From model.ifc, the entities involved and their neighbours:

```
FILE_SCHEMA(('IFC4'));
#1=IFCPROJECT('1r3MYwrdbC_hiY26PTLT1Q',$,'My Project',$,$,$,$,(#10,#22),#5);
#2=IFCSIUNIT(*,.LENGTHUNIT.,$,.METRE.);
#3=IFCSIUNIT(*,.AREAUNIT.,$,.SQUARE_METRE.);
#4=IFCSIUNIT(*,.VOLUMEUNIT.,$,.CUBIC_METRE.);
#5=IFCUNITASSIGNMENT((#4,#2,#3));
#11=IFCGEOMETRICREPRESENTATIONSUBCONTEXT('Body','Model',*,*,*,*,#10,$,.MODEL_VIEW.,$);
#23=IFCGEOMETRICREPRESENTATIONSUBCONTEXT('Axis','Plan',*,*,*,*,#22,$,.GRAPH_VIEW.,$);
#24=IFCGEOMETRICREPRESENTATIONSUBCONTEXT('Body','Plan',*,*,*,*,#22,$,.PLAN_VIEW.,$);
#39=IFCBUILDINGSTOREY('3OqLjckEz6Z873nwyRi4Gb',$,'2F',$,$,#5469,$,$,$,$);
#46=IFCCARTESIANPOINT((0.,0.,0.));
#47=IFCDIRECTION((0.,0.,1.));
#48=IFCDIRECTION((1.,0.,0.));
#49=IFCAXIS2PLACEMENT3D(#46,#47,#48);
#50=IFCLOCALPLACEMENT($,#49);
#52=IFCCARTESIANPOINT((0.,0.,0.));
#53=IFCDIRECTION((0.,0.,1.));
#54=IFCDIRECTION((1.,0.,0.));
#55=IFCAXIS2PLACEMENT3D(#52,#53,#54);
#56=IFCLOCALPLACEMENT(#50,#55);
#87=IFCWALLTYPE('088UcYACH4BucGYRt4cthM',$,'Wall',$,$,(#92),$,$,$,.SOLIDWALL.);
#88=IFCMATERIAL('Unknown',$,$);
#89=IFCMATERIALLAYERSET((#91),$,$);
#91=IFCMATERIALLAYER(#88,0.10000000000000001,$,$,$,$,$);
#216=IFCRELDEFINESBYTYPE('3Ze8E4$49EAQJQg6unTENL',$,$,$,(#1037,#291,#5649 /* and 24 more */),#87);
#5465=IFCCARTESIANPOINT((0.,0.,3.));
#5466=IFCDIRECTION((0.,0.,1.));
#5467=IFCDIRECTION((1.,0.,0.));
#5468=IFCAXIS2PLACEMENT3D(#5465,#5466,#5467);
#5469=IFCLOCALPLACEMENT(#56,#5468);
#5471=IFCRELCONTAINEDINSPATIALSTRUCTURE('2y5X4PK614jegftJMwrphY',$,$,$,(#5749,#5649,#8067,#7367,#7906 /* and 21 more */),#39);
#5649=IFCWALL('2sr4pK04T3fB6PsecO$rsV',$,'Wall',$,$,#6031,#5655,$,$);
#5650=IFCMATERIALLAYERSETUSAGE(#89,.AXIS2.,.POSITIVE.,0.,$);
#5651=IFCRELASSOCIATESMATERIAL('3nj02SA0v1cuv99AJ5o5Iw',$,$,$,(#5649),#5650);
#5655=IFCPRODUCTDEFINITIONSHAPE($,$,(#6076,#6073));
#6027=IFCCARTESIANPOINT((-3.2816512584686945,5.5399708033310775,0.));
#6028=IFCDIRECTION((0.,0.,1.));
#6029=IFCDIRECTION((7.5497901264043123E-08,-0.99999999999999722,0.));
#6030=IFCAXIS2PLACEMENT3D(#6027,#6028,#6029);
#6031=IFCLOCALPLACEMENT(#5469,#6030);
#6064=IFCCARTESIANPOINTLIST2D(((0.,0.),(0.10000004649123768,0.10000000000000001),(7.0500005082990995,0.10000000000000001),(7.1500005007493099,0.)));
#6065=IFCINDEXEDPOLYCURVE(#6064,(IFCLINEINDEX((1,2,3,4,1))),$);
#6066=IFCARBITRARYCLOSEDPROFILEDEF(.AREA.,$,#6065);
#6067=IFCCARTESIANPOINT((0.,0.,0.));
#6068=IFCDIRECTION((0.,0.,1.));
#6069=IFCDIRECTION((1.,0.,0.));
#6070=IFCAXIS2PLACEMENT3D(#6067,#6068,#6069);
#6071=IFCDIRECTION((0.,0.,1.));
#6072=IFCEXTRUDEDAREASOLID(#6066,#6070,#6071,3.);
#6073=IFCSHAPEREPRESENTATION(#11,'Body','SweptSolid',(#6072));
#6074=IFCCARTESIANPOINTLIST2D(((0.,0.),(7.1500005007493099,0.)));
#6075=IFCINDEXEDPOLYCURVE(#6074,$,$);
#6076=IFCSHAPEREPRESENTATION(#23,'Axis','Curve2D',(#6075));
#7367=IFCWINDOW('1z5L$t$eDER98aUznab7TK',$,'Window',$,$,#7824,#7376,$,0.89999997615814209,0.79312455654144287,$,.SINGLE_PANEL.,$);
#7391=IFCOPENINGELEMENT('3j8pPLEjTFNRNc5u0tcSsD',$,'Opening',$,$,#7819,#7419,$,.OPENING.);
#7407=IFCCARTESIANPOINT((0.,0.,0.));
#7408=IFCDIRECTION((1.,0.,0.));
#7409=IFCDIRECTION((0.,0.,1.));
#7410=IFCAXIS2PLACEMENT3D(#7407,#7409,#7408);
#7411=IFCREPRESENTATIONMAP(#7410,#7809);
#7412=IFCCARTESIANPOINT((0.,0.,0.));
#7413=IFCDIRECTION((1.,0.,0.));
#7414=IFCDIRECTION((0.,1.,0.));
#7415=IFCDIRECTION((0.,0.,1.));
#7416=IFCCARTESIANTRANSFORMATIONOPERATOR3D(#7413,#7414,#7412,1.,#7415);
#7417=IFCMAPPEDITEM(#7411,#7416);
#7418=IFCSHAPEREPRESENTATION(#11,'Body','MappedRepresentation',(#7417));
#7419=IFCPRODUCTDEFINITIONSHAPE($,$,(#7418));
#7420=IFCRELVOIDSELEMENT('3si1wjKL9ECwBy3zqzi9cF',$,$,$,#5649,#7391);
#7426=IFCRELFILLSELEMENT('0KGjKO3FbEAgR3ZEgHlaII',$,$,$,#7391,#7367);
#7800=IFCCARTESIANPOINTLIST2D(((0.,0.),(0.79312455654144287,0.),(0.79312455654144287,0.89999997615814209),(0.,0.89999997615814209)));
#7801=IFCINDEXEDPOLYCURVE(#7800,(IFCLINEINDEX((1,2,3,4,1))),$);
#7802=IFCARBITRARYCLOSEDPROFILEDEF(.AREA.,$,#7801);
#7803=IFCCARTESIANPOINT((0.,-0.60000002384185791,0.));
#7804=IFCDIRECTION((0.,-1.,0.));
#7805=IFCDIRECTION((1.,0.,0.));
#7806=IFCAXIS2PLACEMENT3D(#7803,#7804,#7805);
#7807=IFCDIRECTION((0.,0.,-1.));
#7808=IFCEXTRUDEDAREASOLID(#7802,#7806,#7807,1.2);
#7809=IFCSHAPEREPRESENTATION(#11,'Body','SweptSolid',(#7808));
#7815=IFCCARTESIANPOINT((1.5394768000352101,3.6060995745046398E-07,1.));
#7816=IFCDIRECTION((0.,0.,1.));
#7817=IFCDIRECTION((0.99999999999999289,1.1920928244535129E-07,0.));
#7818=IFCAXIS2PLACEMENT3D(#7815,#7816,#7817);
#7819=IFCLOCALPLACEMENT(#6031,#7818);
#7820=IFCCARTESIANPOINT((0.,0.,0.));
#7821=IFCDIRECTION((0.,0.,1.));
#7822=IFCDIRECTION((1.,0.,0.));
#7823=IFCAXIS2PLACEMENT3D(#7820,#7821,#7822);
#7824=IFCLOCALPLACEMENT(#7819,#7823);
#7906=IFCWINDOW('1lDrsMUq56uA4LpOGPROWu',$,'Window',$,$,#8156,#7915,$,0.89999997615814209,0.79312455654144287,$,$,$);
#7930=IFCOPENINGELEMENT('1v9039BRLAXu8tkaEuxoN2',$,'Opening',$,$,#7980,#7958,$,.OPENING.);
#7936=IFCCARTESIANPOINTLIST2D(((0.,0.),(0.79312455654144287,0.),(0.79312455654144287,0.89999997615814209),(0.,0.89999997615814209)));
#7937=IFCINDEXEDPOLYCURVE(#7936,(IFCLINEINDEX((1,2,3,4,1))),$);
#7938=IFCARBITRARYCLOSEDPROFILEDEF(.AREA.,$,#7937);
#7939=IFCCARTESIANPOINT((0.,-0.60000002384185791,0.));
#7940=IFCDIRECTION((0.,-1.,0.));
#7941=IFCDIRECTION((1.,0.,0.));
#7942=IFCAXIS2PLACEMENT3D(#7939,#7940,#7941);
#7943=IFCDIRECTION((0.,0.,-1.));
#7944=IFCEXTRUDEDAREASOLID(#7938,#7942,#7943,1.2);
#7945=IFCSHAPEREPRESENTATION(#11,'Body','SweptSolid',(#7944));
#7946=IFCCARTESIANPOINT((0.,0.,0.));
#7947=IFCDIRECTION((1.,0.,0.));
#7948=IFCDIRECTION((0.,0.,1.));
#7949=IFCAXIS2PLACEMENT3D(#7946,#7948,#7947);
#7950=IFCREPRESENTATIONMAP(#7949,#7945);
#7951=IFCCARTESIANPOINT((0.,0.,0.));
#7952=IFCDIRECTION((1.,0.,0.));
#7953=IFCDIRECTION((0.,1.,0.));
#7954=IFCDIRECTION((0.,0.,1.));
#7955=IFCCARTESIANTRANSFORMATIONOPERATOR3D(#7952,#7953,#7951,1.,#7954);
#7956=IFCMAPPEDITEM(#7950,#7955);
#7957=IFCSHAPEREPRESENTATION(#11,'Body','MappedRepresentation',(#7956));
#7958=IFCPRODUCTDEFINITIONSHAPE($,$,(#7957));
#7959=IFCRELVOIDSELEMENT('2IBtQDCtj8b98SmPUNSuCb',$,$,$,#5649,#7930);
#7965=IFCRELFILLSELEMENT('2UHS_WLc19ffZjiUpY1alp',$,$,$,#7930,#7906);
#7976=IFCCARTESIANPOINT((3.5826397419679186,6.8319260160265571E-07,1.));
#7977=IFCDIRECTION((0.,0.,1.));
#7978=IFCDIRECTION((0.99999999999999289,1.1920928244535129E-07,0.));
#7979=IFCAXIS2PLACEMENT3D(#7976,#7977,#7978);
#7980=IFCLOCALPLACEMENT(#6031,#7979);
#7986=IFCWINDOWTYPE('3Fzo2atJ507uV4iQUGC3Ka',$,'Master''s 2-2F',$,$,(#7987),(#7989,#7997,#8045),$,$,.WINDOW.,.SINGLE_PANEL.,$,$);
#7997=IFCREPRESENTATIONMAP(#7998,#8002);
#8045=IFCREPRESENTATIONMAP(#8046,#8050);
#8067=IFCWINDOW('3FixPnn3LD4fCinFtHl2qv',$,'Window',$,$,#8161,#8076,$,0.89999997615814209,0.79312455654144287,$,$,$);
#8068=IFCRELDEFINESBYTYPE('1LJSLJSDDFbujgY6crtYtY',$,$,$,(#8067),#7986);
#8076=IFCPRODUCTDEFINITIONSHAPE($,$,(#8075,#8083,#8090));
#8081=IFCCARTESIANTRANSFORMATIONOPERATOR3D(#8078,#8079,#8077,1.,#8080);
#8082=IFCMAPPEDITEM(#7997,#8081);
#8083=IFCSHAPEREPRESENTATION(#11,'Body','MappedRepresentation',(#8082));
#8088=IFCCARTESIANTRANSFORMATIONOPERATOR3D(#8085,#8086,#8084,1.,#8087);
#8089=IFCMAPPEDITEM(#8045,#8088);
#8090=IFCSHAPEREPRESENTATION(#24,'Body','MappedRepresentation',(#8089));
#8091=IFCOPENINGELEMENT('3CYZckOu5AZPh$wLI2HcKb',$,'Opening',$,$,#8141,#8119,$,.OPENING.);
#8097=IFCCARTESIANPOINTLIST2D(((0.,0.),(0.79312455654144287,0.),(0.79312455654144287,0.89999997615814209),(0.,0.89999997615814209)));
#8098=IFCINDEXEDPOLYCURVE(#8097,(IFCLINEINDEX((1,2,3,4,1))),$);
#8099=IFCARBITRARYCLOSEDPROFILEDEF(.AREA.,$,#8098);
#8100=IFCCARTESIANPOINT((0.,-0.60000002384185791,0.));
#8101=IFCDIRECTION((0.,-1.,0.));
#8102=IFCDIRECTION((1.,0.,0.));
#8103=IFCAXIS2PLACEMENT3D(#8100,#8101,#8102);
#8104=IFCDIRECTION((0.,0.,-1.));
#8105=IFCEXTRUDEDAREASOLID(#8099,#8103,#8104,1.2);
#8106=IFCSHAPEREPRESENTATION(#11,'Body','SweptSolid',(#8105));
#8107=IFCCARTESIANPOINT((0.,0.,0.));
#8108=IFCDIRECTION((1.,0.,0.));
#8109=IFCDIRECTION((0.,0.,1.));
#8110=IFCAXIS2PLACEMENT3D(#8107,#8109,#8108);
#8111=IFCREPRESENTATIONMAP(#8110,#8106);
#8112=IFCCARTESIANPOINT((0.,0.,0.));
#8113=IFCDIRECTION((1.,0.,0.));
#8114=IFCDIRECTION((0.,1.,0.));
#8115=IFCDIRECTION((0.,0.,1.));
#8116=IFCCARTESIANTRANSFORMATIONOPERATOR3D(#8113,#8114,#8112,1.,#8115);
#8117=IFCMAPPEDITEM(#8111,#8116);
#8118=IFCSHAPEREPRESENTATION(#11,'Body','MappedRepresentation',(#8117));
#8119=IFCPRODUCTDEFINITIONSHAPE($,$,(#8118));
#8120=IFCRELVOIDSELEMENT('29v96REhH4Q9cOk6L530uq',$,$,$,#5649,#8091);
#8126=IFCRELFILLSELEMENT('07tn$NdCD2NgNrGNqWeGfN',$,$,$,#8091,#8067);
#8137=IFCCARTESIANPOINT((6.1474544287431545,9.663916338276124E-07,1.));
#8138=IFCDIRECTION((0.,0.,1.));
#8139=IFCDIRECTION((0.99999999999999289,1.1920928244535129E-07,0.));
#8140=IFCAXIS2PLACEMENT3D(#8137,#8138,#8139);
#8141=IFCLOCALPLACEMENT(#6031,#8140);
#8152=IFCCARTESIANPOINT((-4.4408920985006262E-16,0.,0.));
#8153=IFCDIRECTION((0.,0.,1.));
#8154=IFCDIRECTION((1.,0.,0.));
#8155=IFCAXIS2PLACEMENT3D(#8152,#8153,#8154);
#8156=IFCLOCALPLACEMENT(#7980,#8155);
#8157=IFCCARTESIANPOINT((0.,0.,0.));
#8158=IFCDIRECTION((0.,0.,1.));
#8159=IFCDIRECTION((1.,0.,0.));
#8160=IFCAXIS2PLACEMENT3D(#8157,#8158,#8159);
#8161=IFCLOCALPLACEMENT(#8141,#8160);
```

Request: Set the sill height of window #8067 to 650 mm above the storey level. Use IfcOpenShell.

```python
import numpy as np
import ifcopenshell
import ifcopenshell.api.geometry
import ifcopenshell.geom
import ifcopenshell.util.element
import ifcopenshell.util.placement
import ifcopenshell.util.shape
import ifcopenshell.util.unit

model = ifcopenshell.open("model.ifc")
unit_scale = ifcopenshell.util.unit.calculate_unit_scale(model)

window = model.by_guid("3FixPnn3LD4fCinFtHl2qv")
opening = window.FillsVoids[0].RelatingOpeningElement
storey = ifcopenshell.util.element.get_container(window, ifc_class="IfcBuildingStorey")
level = ifcopenshell.util.placement.get_local_placement(storey.ObjectPlacement)[2, 3]

# The opening's origin need not be at the sill, so measure its lowest point.
shape = ifcopenshell.geom.create_shape(ifcopenshell.geom.settings(), opening)
bottom = ifcopenshell.util.shape.get_shape_bottom_elevation(shape, shape.geometry) / unit_scale
dz = level + 0.65 - bottom

shift = np.array([0.0, 0.0, dz])
# The window is placed relative to its opening, so it follows when the opening moves.
matrix = ifcopenshell.util.placement.get_local_placement(opening.ObjectPlacement)
matrix[:3, 3] += shift
ifcopenshell.api.geometry.edit_object_placement(
    model, product=opening, matrix=matrix, is_si=False, should_transform_children=True
)

print(f"moved by {dz * unit_scale:+.3f} m")

model.write("model-out.ifc")
```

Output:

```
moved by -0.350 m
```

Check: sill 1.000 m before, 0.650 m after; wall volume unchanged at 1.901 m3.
